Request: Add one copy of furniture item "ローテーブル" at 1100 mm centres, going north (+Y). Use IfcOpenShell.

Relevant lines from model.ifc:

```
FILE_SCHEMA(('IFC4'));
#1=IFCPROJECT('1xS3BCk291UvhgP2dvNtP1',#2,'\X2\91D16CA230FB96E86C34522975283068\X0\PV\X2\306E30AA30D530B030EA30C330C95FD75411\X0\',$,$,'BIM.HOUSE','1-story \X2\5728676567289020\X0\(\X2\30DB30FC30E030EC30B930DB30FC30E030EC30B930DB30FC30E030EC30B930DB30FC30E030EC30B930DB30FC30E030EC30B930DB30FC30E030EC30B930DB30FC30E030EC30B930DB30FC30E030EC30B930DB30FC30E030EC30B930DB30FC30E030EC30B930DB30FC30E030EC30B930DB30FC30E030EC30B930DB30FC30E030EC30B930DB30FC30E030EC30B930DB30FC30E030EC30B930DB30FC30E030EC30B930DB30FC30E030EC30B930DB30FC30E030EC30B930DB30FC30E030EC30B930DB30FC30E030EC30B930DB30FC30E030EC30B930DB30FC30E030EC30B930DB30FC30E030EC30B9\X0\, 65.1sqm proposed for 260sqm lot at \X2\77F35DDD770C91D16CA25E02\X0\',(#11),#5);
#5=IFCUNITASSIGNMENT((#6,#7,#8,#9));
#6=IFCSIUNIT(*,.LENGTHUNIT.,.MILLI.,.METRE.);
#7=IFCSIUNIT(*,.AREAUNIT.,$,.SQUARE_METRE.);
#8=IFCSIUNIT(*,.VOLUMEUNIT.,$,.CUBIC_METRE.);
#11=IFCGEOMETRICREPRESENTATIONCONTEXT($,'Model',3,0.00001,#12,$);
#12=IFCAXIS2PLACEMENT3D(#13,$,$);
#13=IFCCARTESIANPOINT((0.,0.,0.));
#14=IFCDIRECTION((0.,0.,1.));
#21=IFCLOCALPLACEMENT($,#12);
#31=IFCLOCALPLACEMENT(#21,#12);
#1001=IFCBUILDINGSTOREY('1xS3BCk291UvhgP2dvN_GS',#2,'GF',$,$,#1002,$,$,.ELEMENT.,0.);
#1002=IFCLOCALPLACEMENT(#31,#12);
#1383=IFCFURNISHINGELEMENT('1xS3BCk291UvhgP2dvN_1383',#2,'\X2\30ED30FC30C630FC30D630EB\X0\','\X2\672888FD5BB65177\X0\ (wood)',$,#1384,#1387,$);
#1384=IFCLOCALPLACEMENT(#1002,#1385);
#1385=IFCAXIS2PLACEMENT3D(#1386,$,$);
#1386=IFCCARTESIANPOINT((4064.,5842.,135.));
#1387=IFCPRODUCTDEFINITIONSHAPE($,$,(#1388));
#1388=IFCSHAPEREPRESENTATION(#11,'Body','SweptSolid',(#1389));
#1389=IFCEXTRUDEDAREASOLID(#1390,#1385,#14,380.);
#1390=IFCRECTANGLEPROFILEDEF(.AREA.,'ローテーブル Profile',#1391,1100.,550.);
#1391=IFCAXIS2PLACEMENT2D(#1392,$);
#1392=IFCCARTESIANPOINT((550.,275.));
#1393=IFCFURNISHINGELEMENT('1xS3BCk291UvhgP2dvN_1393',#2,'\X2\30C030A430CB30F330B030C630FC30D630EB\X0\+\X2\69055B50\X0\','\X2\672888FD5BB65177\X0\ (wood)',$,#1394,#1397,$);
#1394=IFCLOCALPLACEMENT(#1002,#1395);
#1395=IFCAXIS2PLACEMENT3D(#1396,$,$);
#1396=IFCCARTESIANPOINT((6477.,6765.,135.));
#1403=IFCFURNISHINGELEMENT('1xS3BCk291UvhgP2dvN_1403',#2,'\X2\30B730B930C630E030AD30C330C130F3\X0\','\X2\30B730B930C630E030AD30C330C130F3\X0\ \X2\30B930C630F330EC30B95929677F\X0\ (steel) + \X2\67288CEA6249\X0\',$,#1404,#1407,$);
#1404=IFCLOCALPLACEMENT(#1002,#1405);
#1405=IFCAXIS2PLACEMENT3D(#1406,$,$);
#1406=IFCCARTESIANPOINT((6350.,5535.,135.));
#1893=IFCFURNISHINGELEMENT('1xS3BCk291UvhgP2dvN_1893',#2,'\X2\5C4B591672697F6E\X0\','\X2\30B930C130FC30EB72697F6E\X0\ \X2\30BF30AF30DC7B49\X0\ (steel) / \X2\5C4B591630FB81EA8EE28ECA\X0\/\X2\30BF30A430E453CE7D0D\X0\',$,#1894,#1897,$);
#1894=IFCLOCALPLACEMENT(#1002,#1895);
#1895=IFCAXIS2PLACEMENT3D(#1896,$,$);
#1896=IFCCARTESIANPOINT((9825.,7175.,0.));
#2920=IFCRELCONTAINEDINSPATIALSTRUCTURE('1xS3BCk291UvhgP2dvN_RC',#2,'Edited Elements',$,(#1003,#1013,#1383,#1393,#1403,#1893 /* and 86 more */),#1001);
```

```python
import numpy as np
import ifcopenshell
import ifcopenshell.api.geometry
import ifcopenshell.api.root
import ifcopenshell.util.element
import ifcopenshell.util.placement

model = ifcopenshell.open("model.ifc")


def reuse_history(source, copy):
    """copy_class also copies each property set's owner history, people and application; keep the originals."""
    for rel in copy.IsDefinedBy:
        if rel.is_a("IfcRelDefinesByProperties") and (history := rel.RelatingPropertyDefinition.OwnerHistory):
            rel.RelatingPropertyDefinition.OwnerHistory = source.OwnerHistory
            ifcopenshell.util.element.remove_deep2(model, history)


source = model.by_id(1383)
base = ifcopenshell.util.placement.get_local_placement(source.ObjectPlacement)
step = np.array([0.0, 1.0, 0.0]) * 1100.0

for i in range(1, 2):
    copy = ifcopenshell.api.root.copy_class(model, product=source)
    copy.Representation = ifcopenshell.util.element.copy_deep(
        model, source.Representation, exclude=["IfcGeometricRepresentationContext", "IfcRepresentationMap"]
    )
    reuse_history(source, copy)
    matrix = base.copy()
    matrix[:3, 3] += i * step
    print("added at", matrix[:3, 3].round(3) + 0.0)
    ifcopenshell.api.geometry.edit_object_placement(model, product=copy, matrix=matrix, is_si=False)

model.write("model_v2.ifc")
```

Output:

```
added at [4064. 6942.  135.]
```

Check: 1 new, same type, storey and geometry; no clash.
